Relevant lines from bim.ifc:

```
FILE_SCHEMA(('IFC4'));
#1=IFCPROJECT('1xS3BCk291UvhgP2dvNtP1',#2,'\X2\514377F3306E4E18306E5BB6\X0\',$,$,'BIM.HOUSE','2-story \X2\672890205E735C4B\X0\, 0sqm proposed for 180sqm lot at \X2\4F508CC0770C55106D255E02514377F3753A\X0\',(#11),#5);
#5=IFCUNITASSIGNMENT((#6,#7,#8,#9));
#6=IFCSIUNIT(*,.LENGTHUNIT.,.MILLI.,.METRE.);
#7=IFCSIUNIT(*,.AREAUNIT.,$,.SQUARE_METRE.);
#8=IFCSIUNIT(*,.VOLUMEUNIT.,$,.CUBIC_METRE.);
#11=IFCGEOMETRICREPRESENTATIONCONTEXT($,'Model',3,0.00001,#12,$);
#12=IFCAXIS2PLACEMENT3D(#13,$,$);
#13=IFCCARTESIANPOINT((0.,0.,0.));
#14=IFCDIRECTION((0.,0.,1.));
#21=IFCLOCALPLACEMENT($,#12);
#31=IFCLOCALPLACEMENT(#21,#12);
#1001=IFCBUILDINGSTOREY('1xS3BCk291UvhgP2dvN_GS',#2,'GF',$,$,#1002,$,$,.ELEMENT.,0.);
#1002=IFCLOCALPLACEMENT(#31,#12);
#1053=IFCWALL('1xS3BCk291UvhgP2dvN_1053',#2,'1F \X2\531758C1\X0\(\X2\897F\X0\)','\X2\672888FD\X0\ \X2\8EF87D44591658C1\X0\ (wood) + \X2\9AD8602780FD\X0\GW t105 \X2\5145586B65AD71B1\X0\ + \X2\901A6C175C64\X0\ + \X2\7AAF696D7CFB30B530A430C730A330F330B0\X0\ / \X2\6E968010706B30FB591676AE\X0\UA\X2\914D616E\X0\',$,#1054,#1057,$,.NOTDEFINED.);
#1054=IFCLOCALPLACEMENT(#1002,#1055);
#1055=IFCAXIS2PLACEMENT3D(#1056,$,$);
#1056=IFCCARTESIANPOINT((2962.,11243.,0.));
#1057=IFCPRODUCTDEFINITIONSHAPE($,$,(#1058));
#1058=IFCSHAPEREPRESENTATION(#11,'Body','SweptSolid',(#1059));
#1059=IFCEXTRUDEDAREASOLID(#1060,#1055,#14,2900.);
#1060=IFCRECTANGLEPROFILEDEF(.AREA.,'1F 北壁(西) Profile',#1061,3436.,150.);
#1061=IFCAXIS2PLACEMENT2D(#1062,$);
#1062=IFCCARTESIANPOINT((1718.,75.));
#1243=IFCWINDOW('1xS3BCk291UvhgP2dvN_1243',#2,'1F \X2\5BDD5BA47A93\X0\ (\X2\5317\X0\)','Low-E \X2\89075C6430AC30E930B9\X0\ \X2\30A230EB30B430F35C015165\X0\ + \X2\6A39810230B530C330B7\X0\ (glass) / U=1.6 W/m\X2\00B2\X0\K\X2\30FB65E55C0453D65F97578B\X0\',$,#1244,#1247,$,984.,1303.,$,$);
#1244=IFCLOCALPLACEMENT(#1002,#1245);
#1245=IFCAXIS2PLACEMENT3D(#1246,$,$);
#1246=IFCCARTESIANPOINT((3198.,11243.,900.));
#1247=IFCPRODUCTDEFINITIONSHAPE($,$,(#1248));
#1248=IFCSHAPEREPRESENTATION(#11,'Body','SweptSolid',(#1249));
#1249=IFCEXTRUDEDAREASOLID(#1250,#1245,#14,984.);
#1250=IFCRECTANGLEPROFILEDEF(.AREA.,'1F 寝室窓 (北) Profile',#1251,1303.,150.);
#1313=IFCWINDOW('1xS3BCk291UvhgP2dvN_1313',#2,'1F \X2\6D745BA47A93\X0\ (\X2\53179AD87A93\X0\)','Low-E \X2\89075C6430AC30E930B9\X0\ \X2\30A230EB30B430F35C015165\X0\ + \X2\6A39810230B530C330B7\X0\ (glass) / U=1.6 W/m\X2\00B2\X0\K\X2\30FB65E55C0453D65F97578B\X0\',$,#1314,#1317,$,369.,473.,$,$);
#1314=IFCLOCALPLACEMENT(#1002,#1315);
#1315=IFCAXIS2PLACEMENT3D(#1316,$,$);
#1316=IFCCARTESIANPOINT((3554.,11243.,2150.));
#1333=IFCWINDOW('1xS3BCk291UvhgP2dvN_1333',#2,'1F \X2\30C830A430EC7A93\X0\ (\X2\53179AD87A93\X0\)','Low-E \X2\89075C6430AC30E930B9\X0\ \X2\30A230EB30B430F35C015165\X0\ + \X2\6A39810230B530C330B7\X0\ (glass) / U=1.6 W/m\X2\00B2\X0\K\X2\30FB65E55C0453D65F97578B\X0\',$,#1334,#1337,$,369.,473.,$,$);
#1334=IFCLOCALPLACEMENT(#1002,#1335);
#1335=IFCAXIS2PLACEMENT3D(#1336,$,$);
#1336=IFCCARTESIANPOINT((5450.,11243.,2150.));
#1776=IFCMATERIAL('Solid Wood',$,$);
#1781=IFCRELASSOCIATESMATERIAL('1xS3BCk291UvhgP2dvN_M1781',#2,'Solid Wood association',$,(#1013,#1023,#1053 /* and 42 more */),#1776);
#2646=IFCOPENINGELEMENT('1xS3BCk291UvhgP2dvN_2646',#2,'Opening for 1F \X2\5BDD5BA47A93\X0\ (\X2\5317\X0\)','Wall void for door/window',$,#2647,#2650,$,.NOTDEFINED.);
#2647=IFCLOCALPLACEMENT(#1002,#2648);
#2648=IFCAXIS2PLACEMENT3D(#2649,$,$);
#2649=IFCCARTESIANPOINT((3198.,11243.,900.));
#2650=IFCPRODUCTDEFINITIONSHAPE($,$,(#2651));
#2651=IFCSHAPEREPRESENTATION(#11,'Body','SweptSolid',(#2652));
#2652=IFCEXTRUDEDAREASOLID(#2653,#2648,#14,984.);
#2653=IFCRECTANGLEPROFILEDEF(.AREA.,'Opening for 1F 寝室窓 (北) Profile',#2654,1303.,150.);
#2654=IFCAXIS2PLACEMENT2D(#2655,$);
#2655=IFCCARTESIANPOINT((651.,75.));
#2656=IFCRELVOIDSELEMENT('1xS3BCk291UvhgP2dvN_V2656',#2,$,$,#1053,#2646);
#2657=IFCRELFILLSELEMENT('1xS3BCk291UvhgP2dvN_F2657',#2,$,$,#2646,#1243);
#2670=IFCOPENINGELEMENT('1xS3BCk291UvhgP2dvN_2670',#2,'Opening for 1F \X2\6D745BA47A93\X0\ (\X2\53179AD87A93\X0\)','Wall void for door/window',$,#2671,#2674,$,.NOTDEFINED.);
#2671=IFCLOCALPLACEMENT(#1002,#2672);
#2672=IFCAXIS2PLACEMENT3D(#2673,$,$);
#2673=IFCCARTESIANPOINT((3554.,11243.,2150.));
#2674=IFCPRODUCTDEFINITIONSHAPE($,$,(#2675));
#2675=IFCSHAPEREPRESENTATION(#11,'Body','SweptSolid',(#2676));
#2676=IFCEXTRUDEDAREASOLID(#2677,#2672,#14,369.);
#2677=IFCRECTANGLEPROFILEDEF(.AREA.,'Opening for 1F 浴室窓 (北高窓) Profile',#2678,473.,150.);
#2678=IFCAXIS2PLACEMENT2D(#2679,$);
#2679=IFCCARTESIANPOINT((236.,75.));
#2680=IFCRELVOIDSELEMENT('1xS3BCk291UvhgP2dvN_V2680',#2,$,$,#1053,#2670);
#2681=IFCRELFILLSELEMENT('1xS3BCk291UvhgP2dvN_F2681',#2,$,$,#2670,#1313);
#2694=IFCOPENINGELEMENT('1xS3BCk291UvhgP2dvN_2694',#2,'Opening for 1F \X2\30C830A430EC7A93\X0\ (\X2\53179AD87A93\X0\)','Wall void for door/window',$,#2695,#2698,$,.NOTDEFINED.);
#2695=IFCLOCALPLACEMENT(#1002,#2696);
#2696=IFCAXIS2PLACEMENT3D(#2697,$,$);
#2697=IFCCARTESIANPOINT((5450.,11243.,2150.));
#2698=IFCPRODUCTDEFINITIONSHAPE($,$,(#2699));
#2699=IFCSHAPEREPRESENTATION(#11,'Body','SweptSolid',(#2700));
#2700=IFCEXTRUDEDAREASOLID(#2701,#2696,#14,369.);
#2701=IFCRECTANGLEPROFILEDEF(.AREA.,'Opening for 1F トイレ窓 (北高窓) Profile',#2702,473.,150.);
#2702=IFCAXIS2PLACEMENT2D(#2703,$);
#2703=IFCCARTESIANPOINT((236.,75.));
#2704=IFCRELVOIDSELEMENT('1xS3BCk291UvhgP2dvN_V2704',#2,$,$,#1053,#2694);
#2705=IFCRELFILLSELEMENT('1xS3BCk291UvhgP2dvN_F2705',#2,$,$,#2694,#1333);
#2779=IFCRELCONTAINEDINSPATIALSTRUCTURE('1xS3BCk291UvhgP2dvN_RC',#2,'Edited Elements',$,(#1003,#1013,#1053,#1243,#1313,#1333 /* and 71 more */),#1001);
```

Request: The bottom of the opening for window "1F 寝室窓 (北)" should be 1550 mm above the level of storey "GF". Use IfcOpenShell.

```python
import numpy as np
import ifcopenshell
import ifcopenshell.api.geometry
import ifcopenshell.geom
import ifcopenshell.util.element
import ifcopenshell.util.placement
import ifcopenshell.util.shape
import ifcopenshell.util.unit

model = ifcopenshell.open("bim.ifc")
unit_scale = ifcopenshell.util.unit.calculate_unit_scale(model)

window = model.by_guid("1xS3BCk291UvhgP2dvN_1243")
opening = window.FillsVoids[0].RelatingOpeningElement
storey = ifcopenshell.util.element.get_container(window, ifc_class="IfcBuildingStorey")
level = ifcopenshell.util.placement.get_local_placement(storey.ObjectPlacement)[2, 3]

# The opening's origin need not be at the sill, so measure its lowest point.
shape = ifcopenshell.geom.create_shape(ifcopenshell.geom.settings(), opening)
bottom = ifcopenshell.util.shape.get_shape_bottom_elevation(shape, shape.geometry) / unit_scale
dz = level + 1550.0 - bottom

shift = np.array([0.0, 0.0, dz])
# The window is not placed relative to its opening, so move both.
for product in (opening, window):
    matrix = ifcopenshell.util.placement.get_local_placement(product.ObjectPlacement)
    matrix[:3, 3] += shift
    ifcopenshell.api.geometry.edit_object_placement(model, product=product, matrix=matrix, is_si=False)

print(f"moved by {dz * unit_scale:+.3f} m")

model.write("bim-out.ifc")
```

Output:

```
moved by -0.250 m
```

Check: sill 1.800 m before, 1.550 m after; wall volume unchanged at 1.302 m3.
